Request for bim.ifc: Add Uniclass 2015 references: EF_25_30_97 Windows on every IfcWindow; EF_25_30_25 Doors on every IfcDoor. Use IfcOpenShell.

First a look at what the model holds.

```python
import ifcopenshell

model = ifcopenshell.open("bim.ifc")
print(model.schema)
print("classifications:", [c.Name for c in model.by_type("IfcClassification")])
for ifc_class in ("IfcDoor", "IfcRoof", "IfcStair", "IfcWall", "IfcWindow"):
    print(ifc_class, len(model.by_type(ifc_class)))
```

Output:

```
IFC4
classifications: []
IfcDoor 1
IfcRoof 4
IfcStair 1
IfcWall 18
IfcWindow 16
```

```python
import ifcopenshell
import ifcopenshell.api.classification

model = ifcopenshell.open("bim.ifc")

system = ifcopenshell.api.classification.add_classification(model, classification="Uniclass 2015")

codes = {
    "IfcWindow": ("EF_25_30_97", "Windows"),
    "IfcDoor": ("EF_25_30_25", "Doors"),
}
for ifc_class, (code, name) in codes.items():
    products = model.by_type(ifc_class)
    ifcopenshell.api.classification.add_reference(
        model, products=products, classification=system, identification=code, name=name
    )
    print(code, len(products))

model.write("bim-out.ifc")
```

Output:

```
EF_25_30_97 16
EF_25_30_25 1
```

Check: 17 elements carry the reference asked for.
